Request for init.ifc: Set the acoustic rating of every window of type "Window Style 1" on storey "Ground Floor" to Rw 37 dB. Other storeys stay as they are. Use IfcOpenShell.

First a look at what the model holds.

```python
import ifcopenshell
import ifcopenshell.util.element

model = ifcopenshell.open("init.ifc")
print(model.schema)
storey = next(s for s in model.by_type("IfcBuildingStorey") if s.Name == "Ground Floor")
windows = [e for e in ifcopenshell.util.element.get_decomposition(storey) if e.is_a("IfcWindow")]
seen = {}
for e in windows:
    element_type = ifcopenshell.util.element.get_type(e)
    key = (element_type.Name if element_type != e and element_type else None, ifcopenshell.util.element.get_pset(e, "Pset_WindowCommon", "AcousticRating"))
    seen[key] = seen.get(key, 0) + 1
for (name, value), count in sorted(seen.items(), key=str):
    print(count, "x", name, "|", value)
```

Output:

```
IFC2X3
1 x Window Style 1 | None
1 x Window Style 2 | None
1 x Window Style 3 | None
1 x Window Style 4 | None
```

```python
import ifcopenshell
import ifcopenshell.api.pset
import ifcopenshell.util.element

model = ifcopenshell.open("init.ifc")

storey = next(s for s in model.by_type("IfcBuildingStorey") if s.Name == "Ground Floor")
windows = [e for e in ifcopenshell.util.element.get_decomposition(storey) if e.is_a("IfcWindow")]

count = 0
for e in windows:
    element_type = ifcopenshell.util.element.get_type(e)
    if element_type in (None, e) or element_type.Name != "Window Style 1":
        continue
    # add_pset returns the element's existing set when there is one.
    pset = ifcopenshell.api.pset.add_pset(model, product=e, name="Pset_WindowCommon")
    ifcopenshell.api.pset.edit_pset(model, pset=pset, properties={"AcousticRating": "Rw 37 dB"})
    count += 1

print(count, "windows updated")

model.write("init_rev.ifc")
```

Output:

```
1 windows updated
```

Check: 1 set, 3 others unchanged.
